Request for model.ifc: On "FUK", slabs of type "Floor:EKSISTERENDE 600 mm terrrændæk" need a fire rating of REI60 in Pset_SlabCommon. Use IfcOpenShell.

First a look at what the model holds.

```python
import ifcopenshell
import ifcopenshell.util.element

model = ifcopenshell.open("model.ifc")
print(model.schema)
storey = next(s for s in model.by_type("IfcBuildingStorey") if s.Name == "FUK")
slabs = [e for e in ifcopenshell.util.element.get_decomposition(storey) if e.is_a("IfcSlab")]
seen = {}
for e in slabs:
    element_type = ifcopenshell.util.element.get_type(e)
    key = (element_type.Name if element_type != e and element_type else None, ifcopenshell.util.element.get_pset(e, "Pset_SlabCommon", "FireRating"))
    seen[key] = seen.get(key, 0) + 1
for (name, value), count in sorted(seen.items(), key=str):
    print(count, "x", name, "|", value)
```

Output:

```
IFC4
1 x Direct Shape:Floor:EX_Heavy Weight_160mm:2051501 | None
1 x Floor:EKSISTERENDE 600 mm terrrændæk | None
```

```python
import ifcopenshell
import ifcopenshell.api.pset
import ifcopenshell.util.element

model = ifcopenshell.open("model.ifc")

storey = next(s for s in model.by_type("IfcBuildingStorey") if s.Name == "FUK")
slabs = [e for e in ifcopenshell.util.element.get_decomposition(storey) if e.is_a("IfcSlab")]

count = 0
for e in slabs:
    element_type = ifcopenshell.util.element.get_type(e)
    if element_type in (None, e) or element_type.Name != "Floor:EKSISTERENDE 600 mm terrrændæk":
        continue
    # add_pset returns the element's existing set when there is one.
    pset = ifcopenshell.api.pset.add_pset(model, product=e, name="Pset_SlabCommon")
    ifcopenshell.api.pset.edit_pset(model, pset=pset, properties={"FireRating": "REI60"})
    count += 1

print(count, "slabs updated")

model.write("model_edited.ifc")
```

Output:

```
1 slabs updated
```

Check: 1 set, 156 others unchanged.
